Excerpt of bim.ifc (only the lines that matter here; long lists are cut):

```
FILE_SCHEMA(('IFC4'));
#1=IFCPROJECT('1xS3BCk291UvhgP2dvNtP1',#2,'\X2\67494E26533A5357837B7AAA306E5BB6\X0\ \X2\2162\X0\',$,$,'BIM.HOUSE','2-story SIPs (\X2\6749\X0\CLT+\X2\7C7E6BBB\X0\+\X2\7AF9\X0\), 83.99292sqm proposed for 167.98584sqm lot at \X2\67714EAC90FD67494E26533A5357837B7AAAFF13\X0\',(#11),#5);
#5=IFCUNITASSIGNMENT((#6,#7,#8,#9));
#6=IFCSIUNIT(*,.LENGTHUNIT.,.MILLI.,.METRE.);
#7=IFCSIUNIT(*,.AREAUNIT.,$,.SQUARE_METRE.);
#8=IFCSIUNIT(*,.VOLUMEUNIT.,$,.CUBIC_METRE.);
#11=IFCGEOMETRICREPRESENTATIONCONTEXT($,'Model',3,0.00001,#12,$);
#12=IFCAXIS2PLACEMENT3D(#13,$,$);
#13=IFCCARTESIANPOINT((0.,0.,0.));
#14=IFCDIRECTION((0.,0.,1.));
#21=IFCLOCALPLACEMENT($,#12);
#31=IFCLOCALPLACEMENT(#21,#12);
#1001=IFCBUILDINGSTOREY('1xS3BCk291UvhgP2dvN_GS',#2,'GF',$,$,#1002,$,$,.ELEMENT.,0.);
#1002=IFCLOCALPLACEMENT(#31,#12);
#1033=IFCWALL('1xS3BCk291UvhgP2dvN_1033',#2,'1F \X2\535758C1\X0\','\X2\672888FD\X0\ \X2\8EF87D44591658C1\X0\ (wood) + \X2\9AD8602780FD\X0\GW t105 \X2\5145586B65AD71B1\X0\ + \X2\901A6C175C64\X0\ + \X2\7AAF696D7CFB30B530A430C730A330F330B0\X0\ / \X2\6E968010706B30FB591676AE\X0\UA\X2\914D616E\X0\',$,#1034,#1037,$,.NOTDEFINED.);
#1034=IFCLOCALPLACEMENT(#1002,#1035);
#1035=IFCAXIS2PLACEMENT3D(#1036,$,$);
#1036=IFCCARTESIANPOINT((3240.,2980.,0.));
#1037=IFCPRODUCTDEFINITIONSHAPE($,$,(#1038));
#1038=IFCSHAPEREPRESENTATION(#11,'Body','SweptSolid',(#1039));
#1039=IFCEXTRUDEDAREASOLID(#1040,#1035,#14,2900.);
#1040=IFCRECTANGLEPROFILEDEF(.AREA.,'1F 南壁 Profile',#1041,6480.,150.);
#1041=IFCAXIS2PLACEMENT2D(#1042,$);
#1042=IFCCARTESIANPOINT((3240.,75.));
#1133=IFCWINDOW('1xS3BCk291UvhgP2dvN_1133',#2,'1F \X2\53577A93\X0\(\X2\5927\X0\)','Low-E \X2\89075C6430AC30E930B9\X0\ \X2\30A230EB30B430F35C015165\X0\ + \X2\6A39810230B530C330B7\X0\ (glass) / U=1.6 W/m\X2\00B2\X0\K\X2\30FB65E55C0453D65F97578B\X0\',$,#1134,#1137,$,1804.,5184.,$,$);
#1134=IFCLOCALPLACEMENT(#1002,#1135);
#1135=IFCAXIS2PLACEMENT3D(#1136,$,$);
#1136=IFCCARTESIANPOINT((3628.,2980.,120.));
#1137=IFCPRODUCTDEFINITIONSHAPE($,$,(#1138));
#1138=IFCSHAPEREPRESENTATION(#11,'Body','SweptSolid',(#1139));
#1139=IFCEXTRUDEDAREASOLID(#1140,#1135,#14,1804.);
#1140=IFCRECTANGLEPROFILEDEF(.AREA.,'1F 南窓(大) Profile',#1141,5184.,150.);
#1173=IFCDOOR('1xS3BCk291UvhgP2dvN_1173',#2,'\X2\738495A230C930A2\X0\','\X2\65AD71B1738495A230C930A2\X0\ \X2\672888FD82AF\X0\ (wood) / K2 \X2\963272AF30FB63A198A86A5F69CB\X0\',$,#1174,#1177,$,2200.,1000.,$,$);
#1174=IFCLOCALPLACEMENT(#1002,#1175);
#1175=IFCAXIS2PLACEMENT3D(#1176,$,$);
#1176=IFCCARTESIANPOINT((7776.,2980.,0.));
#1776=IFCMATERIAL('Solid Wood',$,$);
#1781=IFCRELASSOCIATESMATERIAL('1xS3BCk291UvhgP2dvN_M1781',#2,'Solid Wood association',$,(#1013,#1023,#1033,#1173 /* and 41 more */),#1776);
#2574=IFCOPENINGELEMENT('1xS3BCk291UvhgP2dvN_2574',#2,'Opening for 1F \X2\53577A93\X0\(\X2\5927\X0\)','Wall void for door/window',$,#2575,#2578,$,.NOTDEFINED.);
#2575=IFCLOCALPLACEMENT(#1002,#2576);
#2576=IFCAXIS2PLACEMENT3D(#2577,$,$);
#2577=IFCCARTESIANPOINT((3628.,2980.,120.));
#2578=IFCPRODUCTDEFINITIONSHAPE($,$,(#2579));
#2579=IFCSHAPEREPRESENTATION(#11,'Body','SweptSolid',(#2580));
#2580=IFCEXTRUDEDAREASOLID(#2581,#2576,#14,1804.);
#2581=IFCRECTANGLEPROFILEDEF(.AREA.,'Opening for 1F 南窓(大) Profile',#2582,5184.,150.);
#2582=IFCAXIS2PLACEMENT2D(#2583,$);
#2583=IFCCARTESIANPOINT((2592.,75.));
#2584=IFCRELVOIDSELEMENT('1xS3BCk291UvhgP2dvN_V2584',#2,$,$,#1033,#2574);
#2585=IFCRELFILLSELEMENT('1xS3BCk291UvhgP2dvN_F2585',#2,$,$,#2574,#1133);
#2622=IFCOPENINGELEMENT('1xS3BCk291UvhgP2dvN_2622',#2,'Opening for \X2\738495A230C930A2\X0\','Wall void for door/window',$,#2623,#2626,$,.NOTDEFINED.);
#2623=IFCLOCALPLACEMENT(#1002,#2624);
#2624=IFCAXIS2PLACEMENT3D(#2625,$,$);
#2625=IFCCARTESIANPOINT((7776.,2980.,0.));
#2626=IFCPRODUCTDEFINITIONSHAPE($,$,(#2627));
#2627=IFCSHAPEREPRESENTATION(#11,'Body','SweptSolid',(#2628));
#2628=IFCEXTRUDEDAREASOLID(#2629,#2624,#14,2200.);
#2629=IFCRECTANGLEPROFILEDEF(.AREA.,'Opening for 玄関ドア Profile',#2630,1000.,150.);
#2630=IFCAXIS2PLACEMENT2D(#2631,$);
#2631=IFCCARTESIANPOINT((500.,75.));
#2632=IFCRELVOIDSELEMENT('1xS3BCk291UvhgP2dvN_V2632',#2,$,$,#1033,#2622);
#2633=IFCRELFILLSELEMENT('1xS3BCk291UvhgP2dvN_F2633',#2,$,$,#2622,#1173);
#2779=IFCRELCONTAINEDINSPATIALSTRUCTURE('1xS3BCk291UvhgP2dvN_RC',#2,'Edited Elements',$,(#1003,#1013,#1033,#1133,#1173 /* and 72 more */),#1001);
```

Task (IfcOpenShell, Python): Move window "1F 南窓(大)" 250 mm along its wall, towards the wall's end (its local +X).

```python
import ifcopenshell
import ifcopenshell.api.geometry
import ifcopenshell.util.placement
import ifcopenshell.util.unit

model = ifcopenshell.open("bim.ifc")
unit_scale = ifcopenshell.util.unit.calculate_unit_scale(model)

window = model.by_guid("1xS3BCk291UvhgP2dvN_1133")
opening = window.FillsVoids[0].RelatingOpeningElement
wall = opening.VoidsElements[0].RelatingBuildingElement

wall_matrix = ifcopenshell.util.placement.get_local_placement(wall.ObjectPlacement)
shift = wall_matrix[:3, 0] * 0.25 / unit_scale
before = ifcopenshell.util.placement.get_local_placement(window.ObjectPlacement)[:3, 3].copy()

# The window is not placed relative to its opening, so move both.
for product in (opening, window):
    matrix = ifcopenshell.util.placement.get_local_placement(product.ObjectPlacement)
    matrix[:3, 3] += shift
    ifcopenshell.api.geometry.edit_object_placement(model, product=product, matrix=matrix, is_si=False)

after = ifcopenshell.util.placement.get_local_placement(window.ObjectPlacement)[:3, 3]
print("window moved by", (after - before).round(3) + 0.0)

model.write("bim_v2.ifc")
```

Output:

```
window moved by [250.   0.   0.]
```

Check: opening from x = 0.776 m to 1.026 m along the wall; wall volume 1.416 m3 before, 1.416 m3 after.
